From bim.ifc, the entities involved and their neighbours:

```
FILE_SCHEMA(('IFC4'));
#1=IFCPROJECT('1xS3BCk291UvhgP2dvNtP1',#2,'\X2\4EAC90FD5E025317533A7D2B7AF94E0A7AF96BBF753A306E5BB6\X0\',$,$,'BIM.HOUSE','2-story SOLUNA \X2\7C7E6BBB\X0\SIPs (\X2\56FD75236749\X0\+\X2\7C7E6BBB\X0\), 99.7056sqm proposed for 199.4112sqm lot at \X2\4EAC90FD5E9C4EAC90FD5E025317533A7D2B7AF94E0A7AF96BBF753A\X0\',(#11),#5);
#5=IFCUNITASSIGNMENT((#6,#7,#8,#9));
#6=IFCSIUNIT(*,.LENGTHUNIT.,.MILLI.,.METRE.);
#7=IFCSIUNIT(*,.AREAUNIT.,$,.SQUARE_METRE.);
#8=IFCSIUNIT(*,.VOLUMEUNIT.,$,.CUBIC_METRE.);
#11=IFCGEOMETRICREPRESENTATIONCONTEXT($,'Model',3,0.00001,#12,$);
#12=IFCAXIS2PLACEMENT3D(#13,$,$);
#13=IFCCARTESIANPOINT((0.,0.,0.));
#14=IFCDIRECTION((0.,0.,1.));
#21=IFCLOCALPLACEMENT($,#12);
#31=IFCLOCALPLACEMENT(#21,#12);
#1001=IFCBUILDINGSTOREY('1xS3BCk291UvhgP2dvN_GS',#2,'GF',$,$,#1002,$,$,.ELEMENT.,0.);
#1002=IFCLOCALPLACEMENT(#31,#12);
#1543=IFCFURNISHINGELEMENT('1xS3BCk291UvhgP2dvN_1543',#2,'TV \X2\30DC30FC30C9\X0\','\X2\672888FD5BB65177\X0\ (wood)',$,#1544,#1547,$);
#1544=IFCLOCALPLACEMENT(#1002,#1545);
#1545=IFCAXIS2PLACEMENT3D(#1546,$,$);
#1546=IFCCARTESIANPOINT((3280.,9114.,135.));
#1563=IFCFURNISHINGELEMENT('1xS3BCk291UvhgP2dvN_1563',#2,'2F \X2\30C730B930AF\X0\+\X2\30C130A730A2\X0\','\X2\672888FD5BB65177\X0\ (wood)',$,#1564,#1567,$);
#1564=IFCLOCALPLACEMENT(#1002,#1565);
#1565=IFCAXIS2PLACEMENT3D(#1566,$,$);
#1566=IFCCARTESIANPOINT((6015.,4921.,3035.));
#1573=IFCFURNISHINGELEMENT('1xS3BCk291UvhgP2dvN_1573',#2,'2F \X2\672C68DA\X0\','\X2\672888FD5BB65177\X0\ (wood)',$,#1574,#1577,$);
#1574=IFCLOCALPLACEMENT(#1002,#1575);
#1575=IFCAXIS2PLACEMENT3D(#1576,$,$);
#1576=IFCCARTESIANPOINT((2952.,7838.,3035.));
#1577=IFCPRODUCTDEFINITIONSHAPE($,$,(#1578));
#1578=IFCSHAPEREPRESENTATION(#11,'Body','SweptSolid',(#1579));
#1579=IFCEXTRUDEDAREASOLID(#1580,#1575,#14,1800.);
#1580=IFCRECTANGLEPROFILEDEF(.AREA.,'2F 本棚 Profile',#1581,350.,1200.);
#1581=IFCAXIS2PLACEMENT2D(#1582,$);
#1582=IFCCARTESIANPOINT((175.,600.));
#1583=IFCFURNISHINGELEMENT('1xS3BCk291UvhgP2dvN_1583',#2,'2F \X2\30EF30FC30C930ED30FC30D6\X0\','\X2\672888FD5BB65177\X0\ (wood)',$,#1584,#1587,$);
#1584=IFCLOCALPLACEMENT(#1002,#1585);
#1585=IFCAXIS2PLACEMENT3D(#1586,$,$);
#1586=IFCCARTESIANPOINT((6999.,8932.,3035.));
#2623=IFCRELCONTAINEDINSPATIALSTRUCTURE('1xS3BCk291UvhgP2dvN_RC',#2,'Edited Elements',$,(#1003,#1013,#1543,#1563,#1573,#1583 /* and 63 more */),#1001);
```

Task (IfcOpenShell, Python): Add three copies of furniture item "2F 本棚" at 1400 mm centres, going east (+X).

```python
import numpy as np
import ifcopenshell
import ifcopenshell.api.geometry
import ifcopenshell.api.root
import ifcopenshell.util.element
import ifcopenshell.util.placement
import ifcopenshell.util.unit

model = ifcopenshell.open("bim.ifc")
unit_scale = ifcopenshell.util.unit.calculate_unit_scale(model)


def reuse_history(source, copy):
    """copy_class also copies each property set's owner history, people and application; keep the originals."""
    for rel in copy.IsDefinedBy:
        if rel.is_a("IfcRelDefinesByProperties") and (history := rel.RelatingPropertyDefinition.OwnerHistory):
            rel.RelatingPropertyDefinition.OwnerHistory = source.OwnerHistory
            ifcopenshell.util.element.remove_deep2(model, history)


source = model.by_guid("1xS3BCk291UvhgP2dvN_1573")
base = ifcopenshell.util.placement.get_local_placement(source.ObjectPlacement)
step = np.array([1.0, 0.0, 0.0]) * 1.4 / unit_scale

for i in range(1, 4):
    copy = ifcopenshell.api.root.copy_class(model, product=source)
    copy.Representation = ifcopenshell.util.element.copy_deep(
        model, source.Representation, exclude=["IfcGeometricRepresentationContext", "IfcRepresentationMap"]
    )
    reuse_history(source, copy)
    matrix = base.copy()
    matrix[:3, 3] += i * step
    print("added at", matrix[:3, 3].round(3) + 0.0)
    ifcopenshell.api.geometry.edit_object_placement(model, product=copy, matrix=matrix, is_si=False)

model.write("bim_v2.ifc")
```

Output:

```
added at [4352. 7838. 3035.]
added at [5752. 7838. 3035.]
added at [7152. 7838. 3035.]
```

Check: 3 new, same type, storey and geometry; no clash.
